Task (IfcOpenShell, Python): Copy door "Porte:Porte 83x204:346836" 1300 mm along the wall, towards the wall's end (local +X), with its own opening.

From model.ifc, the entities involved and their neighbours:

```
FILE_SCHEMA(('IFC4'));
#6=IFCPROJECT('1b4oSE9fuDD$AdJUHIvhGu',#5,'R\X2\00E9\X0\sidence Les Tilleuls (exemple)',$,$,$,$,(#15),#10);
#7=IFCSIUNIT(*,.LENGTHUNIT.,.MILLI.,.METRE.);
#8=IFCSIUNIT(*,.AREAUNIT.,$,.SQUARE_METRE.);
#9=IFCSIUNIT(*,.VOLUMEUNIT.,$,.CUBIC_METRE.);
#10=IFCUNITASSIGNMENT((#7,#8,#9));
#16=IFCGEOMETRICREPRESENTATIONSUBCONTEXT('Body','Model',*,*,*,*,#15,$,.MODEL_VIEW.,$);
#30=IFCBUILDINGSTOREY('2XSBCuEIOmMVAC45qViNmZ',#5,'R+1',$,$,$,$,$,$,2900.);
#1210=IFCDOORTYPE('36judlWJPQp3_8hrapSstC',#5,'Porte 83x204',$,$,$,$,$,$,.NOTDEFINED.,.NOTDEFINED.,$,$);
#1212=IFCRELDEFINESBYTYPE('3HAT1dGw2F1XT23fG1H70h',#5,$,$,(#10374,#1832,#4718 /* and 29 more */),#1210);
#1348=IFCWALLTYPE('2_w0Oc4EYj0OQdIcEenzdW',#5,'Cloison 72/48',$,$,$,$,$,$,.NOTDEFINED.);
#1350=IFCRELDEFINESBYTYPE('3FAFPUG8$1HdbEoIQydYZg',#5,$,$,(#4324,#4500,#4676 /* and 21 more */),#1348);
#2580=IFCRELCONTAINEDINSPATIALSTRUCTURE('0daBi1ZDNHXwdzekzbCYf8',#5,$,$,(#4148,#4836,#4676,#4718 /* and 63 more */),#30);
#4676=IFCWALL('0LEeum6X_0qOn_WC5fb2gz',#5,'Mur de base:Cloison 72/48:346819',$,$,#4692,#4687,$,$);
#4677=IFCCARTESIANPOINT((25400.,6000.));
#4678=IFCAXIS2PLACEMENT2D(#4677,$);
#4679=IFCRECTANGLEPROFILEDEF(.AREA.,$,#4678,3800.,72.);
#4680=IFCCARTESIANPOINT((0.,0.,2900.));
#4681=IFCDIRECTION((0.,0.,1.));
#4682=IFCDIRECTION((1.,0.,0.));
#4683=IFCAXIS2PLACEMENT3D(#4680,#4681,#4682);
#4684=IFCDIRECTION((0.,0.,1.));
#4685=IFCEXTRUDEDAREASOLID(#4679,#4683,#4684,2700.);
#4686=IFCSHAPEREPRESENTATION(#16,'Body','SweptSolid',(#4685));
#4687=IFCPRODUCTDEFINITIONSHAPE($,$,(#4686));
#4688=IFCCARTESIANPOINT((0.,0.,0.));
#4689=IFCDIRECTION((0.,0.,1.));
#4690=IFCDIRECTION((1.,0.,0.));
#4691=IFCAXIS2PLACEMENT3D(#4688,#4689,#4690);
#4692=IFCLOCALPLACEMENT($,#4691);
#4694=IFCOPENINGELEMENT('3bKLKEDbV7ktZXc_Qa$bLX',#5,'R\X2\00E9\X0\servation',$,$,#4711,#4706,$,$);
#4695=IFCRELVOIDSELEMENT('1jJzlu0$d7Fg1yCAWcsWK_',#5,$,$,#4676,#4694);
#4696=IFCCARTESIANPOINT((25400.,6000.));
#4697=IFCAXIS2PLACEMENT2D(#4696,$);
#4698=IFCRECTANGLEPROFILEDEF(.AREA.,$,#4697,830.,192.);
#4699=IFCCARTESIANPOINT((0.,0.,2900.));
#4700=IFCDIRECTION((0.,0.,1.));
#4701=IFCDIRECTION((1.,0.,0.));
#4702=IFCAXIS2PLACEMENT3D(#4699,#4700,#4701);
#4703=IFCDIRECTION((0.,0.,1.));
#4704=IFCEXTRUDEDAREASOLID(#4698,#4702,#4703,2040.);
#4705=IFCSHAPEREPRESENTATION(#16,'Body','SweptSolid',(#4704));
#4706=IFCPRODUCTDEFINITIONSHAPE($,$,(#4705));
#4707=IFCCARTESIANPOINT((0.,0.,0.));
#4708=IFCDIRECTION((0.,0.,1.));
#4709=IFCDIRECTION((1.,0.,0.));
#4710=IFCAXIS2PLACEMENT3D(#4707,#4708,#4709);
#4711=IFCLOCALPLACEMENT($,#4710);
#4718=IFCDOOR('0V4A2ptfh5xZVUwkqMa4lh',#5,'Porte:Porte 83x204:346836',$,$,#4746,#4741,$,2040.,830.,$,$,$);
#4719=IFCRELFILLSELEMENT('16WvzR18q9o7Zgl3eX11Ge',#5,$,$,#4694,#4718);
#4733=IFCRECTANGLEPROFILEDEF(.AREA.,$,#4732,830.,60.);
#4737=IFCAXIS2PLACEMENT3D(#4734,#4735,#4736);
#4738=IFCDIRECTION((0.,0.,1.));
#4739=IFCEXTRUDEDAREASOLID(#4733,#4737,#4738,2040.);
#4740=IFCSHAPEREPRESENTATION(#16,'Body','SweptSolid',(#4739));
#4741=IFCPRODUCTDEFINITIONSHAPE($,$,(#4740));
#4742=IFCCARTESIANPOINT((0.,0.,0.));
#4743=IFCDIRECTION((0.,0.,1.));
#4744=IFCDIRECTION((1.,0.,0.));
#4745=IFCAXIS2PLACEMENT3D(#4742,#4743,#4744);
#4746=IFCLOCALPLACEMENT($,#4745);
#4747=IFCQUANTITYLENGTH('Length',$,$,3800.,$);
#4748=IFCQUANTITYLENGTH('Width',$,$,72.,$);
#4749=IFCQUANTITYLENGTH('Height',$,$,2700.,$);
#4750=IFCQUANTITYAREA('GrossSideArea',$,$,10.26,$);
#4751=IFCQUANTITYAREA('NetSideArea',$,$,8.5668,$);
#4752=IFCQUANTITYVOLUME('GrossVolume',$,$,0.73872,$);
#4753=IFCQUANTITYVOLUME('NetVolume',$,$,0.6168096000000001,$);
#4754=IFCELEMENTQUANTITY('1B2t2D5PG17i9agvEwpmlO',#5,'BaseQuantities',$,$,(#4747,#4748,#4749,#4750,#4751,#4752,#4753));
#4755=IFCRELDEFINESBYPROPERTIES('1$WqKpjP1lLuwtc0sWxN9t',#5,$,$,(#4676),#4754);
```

```python
import ifcopenshell
import ifcopenshell.api.feature
import ifcopenshell.api.geometry
import ifcopenshell.api.pset
import ifcopenshell.api.root
import ifcopenshell.geom
import ifcopenshell.util.element
import ifcopenshell.util.placement
import ifcopenshell.util.shape
import ifcopenshell.util.unit

model = ifcopenshell.open("model.ifc")
unit_scale = ifcopenshell.util.unit.calculate_unit_scale(model)
area_scale = ifcopenshell.util.unit.calculate_unit_scale(model, "AREAUNIT")
volume_scale = ifcopenshell.util.unit.calculate_unit_scale(model, "VOLUMEUNIT")
settings = ifcopenshell.geom.settings()


def volume(element):
    """Net volume in cubic metres, openings subtracted."""
    shape = ifcopenshell.geom.create_shape(settings, element)
    return ifcopenshell.util.shape.get_volume(shape.geometry)


def reuse_history(source, copy):
    """copy_class also copies each property set's owner history, people and application; keep the originals."""
    for rel in copy.IsDefinedBy:
        if rel.is_a("IfcRelDefinesByProperties") and (history := rel.RelatingPropertyDefinition.OwnerHistory):
            rel.RelatingPropertyDefinition.OwnerHistory = source.OwnerHistory
            ifcopenshell.util.element.remove_deep2(model, history)


door = model.by_guid("0V4A2ptfh5xZVUwkqMa4lh")
opening = door.FillsVoids[0].RelatingOpeningElement
wall = opening.VoidsElements[0].RelatingBuildingElement
before = volume(wall)
shift = ifcopenshell.util.placement.get_local_placement(wall.ObjectPlacement)[:3, 0] * 1.3 / unit_scale

# copy_class copies the void relationship, type, container and properties, but no geometry.
new_opening = ifcopenshell.api.root.copy_class(model, product=opening)
new_opening.Representation = ifcopenshell.util.element.copy_deep(
    model, opening.Representation, exclude=["IfcGeometricRepresentationContext", "IfcRepresentationMap"]
)
reuse_history(opening, new_opening)
new_door = ifcopenshell.api.root.copy_class(model, product=door)
new_door.Representation = ifcopenshell.util.element.copy_deep(
    model, door.Representation, exclude=["IfcGeometricRepresentationContext", "IfcRepresentationMap"]
)
new_door.Name = "Porte:Porte 83x204"
reuse_history(door, new_door)
ifcopenshell.api.feature.add_filling(model, opening=new_opening, element=new_door)

for old, new in ((opening, new_opening), (door, new_door)):
    matrix = ifcopenshell.util.placement.get_local_placement(old.ObjectPlacement)
    matrix[:3, 3] += shift
    ifcopenshell.api.geometry.edit_object_placement(model, product=new, matrix=matrix, is_si=False)

after = volume(wall)
thickness = 0.072  # wall thickness in metres

# Update the wall's stored quantities.
qto = model.by_id(ifcopenshell.util.element.get_pset(wall, "BaseQuantities", should_inherit=False)["id"])
ifcopenshell.api.pset.edit_qto(model, qto=qto, properties={
    "NetSideArea": after / thickness / area_scale,
    "NetVolume": after / volume_scale,
})

print(f"wall volume {before:.3f} -> {after:.3f} m3")

model.write("model_edited.ifc")
```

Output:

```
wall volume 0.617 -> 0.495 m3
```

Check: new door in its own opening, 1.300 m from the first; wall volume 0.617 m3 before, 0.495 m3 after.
